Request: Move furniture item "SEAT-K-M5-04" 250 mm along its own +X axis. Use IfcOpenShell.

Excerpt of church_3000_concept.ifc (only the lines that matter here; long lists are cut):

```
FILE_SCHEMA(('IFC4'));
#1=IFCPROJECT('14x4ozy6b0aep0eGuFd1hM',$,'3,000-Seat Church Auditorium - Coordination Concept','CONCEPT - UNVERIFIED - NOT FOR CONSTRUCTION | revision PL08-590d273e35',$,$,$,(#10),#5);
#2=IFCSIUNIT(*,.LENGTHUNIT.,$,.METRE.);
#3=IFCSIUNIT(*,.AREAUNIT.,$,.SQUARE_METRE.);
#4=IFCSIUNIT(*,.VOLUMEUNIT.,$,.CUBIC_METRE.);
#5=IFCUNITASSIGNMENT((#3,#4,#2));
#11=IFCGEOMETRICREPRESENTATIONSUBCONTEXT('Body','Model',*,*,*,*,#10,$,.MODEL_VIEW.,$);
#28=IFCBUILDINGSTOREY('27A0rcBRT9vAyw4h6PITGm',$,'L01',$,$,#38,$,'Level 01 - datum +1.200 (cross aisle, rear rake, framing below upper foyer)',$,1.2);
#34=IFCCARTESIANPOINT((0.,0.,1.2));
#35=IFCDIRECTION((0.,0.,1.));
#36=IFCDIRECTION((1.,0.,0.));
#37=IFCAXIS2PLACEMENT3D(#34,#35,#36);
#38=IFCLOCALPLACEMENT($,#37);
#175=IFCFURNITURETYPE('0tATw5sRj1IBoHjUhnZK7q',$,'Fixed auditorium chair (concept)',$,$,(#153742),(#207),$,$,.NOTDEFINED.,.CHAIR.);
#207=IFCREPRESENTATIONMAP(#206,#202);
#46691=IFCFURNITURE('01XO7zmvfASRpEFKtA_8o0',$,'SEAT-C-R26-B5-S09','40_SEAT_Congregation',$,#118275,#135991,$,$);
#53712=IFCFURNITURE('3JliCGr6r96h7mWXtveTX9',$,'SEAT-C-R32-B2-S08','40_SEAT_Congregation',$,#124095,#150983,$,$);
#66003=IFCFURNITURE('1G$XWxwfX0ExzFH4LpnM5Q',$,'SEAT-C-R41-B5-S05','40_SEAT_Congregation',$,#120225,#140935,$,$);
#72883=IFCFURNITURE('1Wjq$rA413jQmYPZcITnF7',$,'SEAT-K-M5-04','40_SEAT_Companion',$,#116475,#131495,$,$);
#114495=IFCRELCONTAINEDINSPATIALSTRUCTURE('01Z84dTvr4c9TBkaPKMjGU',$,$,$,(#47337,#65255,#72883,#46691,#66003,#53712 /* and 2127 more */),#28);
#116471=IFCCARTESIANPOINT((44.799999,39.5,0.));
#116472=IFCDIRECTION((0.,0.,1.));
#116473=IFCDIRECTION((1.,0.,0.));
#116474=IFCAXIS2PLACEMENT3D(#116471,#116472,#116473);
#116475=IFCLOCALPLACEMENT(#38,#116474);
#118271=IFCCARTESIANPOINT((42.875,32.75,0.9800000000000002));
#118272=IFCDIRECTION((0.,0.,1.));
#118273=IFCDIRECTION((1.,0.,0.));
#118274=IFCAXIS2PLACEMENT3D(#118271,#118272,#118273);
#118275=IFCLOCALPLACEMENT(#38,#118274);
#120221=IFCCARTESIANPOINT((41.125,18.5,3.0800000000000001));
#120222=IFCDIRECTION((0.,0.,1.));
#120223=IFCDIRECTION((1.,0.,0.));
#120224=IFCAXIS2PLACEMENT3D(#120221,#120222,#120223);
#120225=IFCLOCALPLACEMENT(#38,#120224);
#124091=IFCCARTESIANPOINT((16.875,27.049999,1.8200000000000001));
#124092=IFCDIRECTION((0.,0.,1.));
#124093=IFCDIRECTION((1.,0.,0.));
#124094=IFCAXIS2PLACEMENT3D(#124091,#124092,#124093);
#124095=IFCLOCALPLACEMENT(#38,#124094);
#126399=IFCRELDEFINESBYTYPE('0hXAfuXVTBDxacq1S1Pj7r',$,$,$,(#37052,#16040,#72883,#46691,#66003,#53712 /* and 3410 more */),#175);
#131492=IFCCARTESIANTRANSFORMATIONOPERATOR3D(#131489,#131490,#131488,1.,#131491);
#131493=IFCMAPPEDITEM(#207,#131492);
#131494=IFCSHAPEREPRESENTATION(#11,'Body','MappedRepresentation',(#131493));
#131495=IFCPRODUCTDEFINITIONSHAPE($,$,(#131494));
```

```python
import ifcopenshell
import ifcopenshell.api.geometry
import ifcopenshell.util.placement
import ifcopenshell.util.unit

model = ifcopenshell.open("church_3000_concept.ifc")
unit_scale = ifcopenshell.util.unit.calculate_unit_scale(model)

item = model.by_guid("1Wjq$rA413jQmYPZcITnF7")
matrix = ifcopenshell.util.placement.get_local_placement(item.ObjectPlacement)
matrix[:3, 3] += matrix[:3, 0] * 0.25 / unit_scale
ifcopenshell.api.geometry.edit_object_placement(model, product=item, matrix=matrix, is_si=False)

print(ifcopenshell.util.placement.get_local_placement(item.ObjectPlacement).round(3) + 0.0)

model.write("church_3000_concept_rev.ifc")
```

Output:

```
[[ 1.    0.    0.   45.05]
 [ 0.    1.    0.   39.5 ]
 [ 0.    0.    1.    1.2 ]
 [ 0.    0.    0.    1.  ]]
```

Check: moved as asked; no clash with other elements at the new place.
